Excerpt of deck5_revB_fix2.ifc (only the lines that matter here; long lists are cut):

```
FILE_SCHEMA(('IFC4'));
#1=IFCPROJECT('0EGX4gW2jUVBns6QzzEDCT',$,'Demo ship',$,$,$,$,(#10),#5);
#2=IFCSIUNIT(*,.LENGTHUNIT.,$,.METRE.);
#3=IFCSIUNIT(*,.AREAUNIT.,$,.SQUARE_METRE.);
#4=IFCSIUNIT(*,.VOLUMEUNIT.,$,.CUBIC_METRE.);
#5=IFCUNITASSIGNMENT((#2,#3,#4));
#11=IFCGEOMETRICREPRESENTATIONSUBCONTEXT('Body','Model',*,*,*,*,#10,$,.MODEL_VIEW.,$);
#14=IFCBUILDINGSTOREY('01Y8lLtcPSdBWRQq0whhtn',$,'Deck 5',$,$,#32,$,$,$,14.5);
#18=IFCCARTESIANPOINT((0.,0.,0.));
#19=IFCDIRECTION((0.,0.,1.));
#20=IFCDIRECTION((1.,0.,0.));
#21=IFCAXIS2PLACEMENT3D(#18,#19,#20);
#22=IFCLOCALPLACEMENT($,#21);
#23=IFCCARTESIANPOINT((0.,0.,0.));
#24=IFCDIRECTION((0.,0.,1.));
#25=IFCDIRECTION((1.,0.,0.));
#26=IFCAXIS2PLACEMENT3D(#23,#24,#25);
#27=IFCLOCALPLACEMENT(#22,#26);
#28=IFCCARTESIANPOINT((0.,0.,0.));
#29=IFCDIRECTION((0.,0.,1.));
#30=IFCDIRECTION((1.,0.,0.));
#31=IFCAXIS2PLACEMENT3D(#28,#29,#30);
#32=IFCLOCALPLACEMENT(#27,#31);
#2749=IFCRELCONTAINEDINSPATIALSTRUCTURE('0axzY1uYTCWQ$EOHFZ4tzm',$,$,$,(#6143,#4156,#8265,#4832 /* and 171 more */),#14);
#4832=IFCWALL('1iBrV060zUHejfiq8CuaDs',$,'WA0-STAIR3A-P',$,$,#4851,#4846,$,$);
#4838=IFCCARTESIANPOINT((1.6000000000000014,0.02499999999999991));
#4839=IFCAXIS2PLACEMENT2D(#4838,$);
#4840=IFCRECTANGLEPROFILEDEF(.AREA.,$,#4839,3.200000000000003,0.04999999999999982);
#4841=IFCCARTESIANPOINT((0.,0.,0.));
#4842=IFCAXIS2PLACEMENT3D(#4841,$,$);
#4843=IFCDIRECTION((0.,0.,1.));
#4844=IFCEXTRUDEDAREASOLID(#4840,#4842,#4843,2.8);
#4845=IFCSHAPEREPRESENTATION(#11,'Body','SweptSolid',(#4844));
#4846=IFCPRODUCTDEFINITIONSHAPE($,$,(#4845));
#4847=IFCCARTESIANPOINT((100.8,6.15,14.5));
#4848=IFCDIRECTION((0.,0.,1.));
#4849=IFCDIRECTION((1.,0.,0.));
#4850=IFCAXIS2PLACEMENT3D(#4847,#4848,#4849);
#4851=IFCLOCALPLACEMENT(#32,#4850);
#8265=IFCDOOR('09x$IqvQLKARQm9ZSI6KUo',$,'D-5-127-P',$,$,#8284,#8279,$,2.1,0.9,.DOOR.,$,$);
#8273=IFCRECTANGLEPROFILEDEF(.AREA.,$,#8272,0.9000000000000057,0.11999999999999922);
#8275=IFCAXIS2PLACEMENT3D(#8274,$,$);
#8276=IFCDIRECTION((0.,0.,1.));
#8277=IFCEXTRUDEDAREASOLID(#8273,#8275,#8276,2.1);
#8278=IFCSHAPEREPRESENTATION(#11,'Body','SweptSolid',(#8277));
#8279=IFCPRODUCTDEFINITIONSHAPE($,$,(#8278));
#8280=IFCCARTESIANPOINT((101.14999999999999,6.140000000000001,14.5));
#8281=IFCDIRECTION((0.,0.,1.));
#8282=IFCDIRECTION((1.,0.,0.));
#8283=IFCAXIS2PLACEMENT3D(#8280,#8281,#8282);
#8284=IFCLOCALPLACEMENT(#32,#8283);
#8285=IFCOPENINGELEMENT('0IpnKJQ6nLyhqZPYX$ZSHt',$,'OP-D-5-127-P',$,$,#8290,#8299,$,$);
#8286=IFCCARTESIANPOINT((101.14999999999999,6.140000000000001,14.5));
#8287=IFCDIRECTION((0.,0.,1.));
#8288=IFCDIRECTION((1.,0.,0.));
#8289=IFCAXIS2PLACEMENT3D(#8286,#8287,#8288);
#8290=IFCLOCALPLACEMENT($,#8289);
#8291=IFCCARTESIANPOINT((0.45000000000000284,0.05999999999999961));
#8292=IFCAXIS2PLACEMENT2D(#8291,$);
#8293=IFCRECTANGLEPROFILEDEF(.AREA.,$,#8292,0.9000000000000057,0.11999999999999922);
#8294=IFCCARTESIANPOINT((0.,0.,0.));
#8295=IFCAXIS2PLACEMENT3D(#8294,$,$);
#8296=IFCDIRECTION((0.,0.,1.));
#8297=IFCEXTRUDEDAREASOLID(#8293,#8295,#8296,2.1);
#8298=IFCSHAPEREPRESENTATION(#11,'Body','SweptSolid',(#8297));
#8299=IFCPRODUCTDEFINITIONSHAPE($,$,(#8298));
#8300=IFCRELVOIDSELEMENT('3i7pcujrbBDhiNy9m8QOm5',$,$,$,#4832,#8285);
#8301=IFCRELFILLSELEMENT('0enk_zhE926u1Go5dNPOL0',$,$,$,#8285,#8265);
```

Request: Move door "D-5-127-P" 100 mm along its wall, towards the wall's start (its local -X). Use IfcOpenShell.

```python
import ifcopenshell
import ifcopenshell.api.geometry
import ifcopenshell.util.placement

model = ifcopenshell.open("deck5_revB_fix2.ifc")

door = model.by_guid("09x$IqvQLKARQm9ZSI6KUo")
opening = door.FillsVoids[0].RelatingOpeningElement
wall = opening.VoidsElements[0].RelatingBuildingElement

wall_matrix = ifcopenshell.util.placement.get_local_placement(wall.ObjectPlacement)
shift = wall_matrix[:3, 0] * -0.1
before = ifcopenshell.util.placement.get_local_placement(door.ObjectPlacement)[:3, 3].copy()

# The door is not placed relative to its opening, so move both.
for product in (opening, door):
    matrix = ifcopenshell.util.placement.get_local_placement(product.ObjectPlacement)
    matrix[:3, 3] += shift
    ifcopenshell.api.geometry.edit_object_placement(model, product=product, matrix=matrix, is_si=False)

after = ifcopenshell.util.placement.get_local_placement(door.ObjectPlacement)[:3, 3]
print("door moved by", (after - before).round(3) + 0.0)

model.write("deck5_revB_fix2_rev.ifc")
```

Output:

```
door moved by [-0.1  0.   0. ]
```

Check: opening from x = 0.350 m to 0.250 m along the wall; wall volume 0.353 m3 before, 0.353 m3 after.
